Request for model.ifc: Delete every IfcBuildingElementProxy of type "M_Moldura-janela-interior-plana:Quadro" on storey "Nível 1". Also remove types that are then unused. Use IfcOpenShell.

First a look at what the model holds.

```python
import ifcopenshell
import ifcopenshell.util.element

model = ifcopenshell.open("model.ifc")
print(model.schema)
storey = next(s for s in model.by_type("IfcBuildingStorey") if s.Name == "Nível 1")
proxies = [e for e in ifcopenshell.util.element.get_decomposition(storey) if e.is_a("IfcBuildingElementProxy")]
seen = {}
for e in proxies:
    element_type = ifcopenshell.util.element.get_type(e)
    name = element_type.Name if element_type not in (None, e) else None
    seen[name] = seen.get(name, 0) + 1
for name, count in sorted(seen.items(), key=str):
    print(count, "x", name)
```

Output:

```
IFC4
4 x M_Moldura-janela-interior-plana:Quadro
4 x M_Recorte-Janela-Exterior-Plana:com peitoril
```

```python
import ifcopenshell
import ifcopenshell.api.root
import ifcopenshell.util.element

model = ifcopenshell.open("model.ifc")

storey = next(s for s in model.by_type("IfcBuildingStorey") if s.Name == "Nível 1")
proxies = [e for e in ifcopenshell.util.element.get_decomposition(storey) if e.is_a("IfcBuildingElementProxy")]
targets = [e for e in proxies if (t := ifcopenshell.util.element.get_type(e)) not in (None, e) and t.Name == "M_Moldura-janela-interior-plana:Quadro"]
types = {ifcopenshell.util.element.get_type(e) for e in targets} - {None, *targets}

for e in targets:
    ifcopenshell.api.root.remove_product(model, product=e)
print(len(targets), "removed")

unused = [t for t in types if not ifcopenshell.util.element.get_types(t)]
for t in unused:
    ifcopenshell.api.root.remove_product(model, product=t)
print(len(unused), "unused types removed")

model.write("model_rev.ifc")
```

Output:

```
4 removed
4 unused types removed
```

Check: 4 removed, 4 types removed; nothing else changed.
